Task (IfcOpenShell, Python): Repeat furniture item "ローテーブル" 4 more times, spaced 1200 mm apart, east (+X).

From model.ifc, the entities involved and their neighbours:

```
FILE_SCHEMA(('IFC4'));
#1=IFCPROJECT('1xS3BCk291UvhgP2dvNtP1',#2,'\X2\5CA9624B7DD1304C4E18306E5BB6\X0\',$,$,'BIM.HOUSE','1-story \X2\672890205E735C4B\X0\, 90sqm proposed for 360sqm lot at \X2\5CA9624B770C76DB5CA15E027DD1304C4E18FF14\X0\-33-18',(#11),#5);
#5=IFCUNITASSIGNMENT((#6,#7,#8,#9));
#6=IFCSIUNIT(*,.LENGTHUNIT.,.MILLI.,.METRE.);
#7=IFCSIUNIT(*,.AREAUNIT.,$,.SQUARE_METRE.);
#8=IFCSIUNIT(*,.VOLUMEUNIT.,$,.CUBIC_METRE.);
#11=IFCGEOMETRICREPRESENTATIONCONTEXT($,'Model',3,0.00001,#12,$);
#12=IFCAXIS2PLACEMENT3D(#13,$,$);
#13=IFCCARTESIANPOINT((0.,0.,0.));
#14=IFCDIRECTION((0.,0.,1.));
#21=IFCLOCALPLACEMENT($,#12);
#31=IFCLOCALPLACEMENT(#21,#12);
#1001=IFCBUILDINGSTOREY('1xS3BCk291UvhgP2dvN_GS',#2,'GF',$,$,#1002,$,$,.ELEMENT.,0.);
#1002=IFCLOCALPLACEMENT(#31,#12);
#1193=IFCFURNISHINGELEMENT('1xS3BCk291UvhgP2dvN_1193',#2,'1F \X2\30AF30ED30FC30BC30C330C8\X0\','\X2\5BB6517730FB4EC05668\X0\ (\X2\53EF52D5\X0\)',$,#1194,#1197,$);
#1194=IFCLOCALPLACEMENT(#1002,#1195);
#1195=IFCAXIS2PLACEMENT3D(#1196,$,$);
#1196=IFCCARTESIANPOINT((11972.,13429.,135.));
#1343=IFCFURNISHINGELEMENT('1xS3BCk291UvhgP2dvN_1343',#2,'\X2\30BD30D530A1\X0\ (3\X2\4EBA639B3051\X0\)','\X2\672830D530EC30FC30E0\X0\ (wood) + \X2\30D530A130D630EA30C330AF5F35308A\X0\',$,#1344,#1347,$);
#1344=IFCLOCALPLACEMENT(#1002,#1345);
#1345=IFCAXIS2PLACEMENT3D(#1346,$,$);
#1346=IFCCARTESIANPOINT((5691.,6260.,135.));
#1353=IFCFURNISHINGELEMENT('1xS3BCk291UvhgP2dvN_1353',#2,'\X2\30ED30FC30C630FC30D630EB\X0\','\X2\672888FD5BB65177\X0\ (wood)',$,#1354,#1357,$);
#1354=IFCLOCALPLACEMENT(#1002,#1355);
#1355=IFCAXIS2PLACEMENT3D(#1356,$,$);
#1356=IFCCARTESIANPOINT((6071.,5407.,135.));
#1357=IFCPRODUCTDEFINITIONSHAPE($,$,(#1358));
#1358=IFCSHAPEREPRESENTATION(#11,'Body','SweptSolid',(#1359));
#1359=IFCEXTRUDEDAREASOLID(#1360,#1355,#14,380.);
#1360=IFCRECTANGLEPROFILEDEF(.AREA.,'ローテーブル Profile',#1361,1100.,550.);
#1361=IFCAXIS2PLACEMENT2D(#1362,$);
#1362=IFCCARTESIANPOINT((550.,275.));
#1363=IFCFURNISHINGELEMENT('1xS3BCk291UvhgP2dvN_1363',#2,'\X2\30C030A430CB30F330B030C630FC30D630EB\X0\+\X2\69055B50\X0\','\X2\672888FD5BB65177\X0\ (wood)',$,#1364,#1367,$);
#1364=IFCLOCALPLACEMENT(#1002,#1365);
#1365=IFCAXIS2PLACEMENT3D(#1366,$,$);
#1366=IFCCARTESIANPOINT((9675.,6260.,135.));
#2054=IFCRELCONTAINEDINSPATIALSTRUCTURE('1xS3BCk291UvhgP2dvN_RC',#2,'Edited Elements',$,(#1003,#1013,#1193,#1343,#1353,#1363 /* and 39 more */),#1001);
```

```python
import numpy as np
import ifcopenshell
import ifcopenshell.api.geometry
import ifcopenshell.api.root
import ifcopenshell.util.element
import ifcopenshell.util.placement
import ifcopenshell.util.unit

model = ifcopenshell.open("model.ifc")
unit_scale = ifcopenshell.util.unit.calculate_unit_scale(model)


def reuse_history(source, copy):
    """copy_class also copies each property set's owner history, people and application; keep the originals."""
    for rel in copy.IsDefinedBy:
        if rel.is_a("IfcRelDefinesByProperties") and (history := rel.RelatingPropertyDefinition.OwnerHistory):
            rel.RelatingPropertyDefinition.OwnerHistory = source.OwnerHistory
            ifcopenshell.util.element.remove_deep2(model, history)


source = model.by_guid("1xS3BCk291UvhgP2dvN_1353")
base = ifcopenshell.util.placement.get_local_placement(source.ObjectPlacement)
step = np.array([1.0, 0.0, 0.0]) * 1.2 / unit_scale

for i in range(1, 5):
    copy = ifcopenshell.api.root.copy_class(model, product=source)
    copy.Representation = ifcopenshell.util.element.copy_deep(
        model, source.Representation, exclude=["IfcGeometricRepresentationContext", "IfcRepresentationMap"]
    )
    reuse_history(source, copy)
    matrix = base.copy()
    matrix[:3, 3] += i * step
    print("added at", matrix[:3, 3].round(3) + 0.0)
    ifcopenshell.api.geometry.edit_object_placement(model, product=copy, matrix=matrix, is_si=False)

model.write("model_updated.ifc")
```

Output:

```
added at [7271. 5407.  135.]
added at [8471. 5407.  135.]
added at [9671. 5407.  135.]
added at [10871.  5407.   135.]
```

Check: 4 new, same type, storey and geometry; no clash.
